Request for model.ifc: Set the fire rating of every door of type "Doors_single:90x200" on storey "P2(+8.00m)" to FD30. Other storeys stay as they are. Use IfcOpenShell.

First a look at what the model holds.

```python
import ifcopenshell
import ifcopenshell.util.element

model = ifcopenshell.open("model.ifc")
print(model.schema)
storey = next(s for s in model.by_type("IfcBuildingStorey") if s.Name == "P2(+8.00m)")
doors = [e for e in ifcopenshell.util.element.get_decomposition(storey) if e.is_a("IfcDoor")]
seen = {}
for e in doors:
    element_type = ifcopenshell.util.element.get_type(e)
    key = (element_type.Name if element_type != e and element_type else None, ifcopenshell.util.element.get_pset(e, "Pset_DoorCommon", "FireRating"))
    seen[key] = seen.get(key, 0) + 1
for (name, value), count in sorted(seen.items(), key=str):
    print(count, "x", name, "|", value)
```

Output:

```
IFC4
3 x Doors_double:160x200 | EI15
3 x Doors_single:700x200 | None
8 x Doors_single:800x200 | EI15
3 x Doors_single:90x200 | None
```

```python
import ifcopenshell
import ifcopenshell.api.pset
import ifcopenshell.util.element

model = ifcopenshell.open("model.ifc")

storey = next(s for s in model.by_type("IfcBuildingStorey") if s.Name == "P2(+8.00m)")
doors = [e for e in ifcopenshell.util.element.get_decomposition(storey) if e.is_a("IfcDoor")]

count = 0
for e in doors:
    element_type = ifcopenshell.util.element.get_type(e)
    if element_type in (None, e) or element_type.Name != "Doors_single:90x200":
        continue
    # add_pset returns the element's existing set when there is one.
    pset = ifcopenshell.api.pset.add_pset(model, product=e, name="Pset_DoorCommon")
    ifcopenshell.api.pset.edit_pset(model, pset=pset, properties={"FireRating": "FD30"})
    count += 1

print(count, "doors updated")

model.write("model-out.ifc")
```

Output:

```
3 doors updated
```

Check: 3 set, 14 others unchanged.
